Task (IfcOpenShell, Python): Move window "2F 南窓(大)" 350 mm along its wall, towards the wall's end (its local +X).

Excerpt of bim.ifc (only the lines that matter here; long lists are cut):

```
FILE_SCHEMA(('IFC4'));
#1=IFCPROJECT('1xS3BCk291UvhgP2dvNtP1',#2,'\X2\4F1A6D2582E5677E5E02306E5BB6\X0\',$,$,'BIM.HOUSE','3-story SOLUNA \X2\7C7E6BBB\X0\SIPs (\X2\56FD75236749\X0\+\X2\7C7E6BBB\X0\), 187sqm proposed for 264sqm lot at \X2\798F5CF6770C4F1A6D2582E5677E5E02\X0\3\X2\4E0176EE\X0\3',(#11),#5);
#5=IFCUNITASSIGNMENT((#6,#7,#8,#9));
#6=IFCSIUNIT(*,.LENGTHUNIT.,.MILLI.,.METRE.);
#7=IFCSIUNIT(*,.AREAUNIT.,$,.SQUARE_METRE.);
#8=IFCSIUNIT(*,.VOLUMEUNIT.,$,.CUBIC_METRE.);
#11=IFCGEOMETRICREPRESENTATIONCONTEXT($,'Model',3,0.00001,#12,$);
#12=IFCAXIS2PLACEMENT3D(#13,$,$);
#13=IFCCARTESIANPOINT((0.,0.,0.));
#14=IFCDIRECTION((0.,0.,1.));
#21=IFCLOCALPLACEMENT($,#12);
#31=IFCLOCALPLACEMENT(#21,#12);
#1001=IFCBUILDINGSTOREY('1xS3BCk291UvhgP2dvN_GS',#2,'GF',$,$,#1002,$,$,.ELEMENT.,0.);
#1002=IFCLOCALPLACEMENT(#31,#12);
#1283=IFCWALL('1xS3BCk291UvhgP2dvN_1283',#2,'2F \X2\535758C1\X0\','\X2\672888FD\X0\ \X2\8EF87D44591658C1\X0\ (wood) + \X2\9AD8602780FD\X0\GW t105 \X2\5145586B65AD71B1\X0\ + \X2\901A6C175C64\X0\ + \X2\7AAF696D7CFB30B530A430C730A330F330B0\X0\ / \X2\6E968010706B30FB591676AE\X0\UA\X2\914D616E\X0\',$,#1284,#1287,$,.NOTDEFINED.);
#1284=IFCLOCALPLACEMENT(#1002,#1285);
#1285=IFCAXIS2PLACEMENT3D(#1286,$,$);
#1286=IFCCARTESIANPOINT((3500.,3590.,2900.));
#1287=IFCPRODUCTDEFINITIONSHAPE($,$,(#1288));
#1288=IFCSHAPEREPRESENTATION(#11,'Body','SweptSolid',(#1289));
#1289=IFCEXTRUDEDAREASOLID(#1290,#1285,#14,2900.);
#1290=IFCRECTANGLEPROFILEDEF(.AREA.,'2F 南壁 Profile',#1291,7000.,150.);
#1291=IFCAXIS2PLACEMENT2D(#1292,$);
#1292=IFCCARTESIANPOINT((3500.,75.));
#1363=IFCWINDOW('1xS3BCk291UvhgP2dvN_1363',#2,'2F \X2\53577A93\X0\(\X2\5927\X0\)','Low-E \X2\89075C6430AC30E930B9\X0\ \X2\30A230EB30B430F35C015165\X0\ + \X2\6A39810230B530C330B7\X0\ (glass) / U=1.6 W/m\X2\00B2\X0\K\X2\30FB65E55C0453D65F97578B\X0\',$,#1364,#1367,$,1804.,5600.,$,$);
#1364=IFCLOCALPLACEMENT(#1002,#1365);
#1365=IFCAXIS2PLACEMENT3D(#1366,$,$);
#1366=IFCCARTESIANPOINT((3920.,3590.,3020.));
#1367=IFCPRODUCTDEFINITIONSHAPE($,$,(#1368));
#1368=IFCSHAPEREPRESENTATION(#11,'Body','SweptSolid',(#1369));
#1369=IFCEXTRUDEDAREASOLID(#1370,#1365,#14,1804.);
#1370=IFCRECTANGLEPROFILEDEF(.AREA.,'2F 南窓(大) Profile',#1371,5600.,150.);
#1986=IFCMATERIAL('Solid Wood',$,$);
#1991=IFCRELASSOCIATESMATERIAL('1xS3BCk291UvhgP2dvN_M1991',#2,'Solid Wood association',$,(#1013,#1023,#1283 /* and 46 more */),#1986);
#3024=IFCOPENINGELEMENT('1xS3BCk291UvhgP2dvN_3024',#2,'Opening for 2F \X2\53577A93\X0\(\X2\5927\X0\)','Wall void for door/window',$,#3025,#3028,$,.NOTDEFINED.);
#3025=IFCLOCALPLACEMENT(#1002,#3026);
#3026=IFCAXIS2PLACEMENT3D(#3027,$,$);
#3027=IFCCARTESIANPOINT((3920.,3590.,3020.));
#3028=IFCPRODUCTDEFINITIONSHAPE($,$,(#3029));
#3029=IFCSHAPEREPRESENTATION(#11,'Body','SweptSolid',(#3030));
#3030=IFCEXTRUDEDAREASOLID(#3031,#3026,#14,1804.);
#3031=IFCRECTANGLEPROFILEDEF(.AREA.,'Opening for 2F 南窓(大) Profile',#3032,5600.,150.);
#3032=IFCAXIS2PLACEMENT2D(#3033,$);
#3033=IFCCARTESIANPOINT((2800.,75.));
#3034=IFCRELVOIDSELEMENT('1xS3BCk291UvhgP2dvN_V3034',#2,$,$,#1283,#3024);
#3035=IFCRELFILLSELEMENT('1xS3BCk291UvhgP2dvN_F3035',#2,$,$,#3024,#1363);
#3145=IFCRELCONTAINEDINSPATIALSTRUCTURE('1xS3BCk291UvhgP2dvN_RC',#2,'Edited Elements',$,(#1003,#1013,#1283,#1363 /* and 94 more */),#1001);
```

```python
import ifcopenshell
import ifcopenshell.api.geometry
import ifcopenshell.util.placement
import ifcopenshell.util.unit

model = ifcopenshell.open("bim.ifc")
unit_scale = ifcopenshell.util.unit.calculate_unit_scale(model)

window = model.by_guid("1xS3BCk291UvhgP2dvN_1363")
opening = window.FillsVoids[0].RelatingOpeningElement
wall = opening.VoidsElements[0].RelatingBuildingElement

wall_matrix = ifcopenshell.util.placement.get_local_placement(wall.ObjectPlacement)
shift = wall_matrix[:3, 0] * 0.35 / unit_scale
before = ifcopenshell.util.placement.get_local_placement(window.ObjectPlacement)[:3, 3].copy()

# The window is not placed relative to its opening, so move both.
for product in (opening, window):
    matrix = ifcopenshell.util.placement.get_local_placement(product.ObjectPlacement)
    matrix[:3, 3] += shift
    ifcopenshell.api.geometry.edit_object_placement(model, product=product, matrix=matrix, is_si=False)

after = ifcopenshell.util.placement.get_local_placement(window.ObjectPlacement)[:3, 3]
print("window moved by", (after - before).round(3) + 0.0)

model.write("bim_edited.ifc")
```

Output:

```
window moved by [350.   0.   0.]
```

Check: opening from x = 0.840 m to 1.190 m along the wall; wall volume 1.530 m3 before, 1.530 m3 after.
